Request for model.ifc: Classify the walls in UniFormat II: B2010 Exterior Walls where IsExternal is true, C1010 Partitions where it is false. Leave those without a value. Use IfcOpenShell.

First a look at what the model holds.

```python
import ifcopenshell
import ifcopenshell.util.element

model = ifcopenshell.open("model.ifc")
print(model.schema)
print("classifications:", [c.Name for c in model.by_type("IfcClassification")])
values = [ifcopenshell.util.element.get_pset(e, "Pset_WallCommon", "IsExternal") for e in model.by_type("IfcWall")]
for value in (True, False, None):
    print("IsExternal", value, values.count(value))
```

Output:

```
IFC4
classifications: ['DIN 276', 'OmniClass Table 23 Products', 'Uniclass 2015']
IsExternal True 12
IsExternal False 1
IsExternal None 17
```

```python
import ifcopenshell
import ifcopenshell.api.classification
import ifcopenshell.util.element

model = ifcopenshell.open("model.ifc")

system = ifcopenshell.api.classification.add_classification(model, classification="UniFormat II")

walls = model.by_type("IfcWall")
external = {e: ifcopenshell.util.element.get_pset(e, "Pset_WallCommon", "IsExternal") for e in walls}
for flag, code, name in ((True, "B2010", "Exterior Walls"), (False, "C1010", "Partitions")):
    products = [e for e in walls if external[e] is flag]
    ifcopenshell.api.classification.add_reference(
        model, products=products, classification=system, identification=code, name=name
    )
    print(code, len(products))

model.write("model_rev.ifc")
```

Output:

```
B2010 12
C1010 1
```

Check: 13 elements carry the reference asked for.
